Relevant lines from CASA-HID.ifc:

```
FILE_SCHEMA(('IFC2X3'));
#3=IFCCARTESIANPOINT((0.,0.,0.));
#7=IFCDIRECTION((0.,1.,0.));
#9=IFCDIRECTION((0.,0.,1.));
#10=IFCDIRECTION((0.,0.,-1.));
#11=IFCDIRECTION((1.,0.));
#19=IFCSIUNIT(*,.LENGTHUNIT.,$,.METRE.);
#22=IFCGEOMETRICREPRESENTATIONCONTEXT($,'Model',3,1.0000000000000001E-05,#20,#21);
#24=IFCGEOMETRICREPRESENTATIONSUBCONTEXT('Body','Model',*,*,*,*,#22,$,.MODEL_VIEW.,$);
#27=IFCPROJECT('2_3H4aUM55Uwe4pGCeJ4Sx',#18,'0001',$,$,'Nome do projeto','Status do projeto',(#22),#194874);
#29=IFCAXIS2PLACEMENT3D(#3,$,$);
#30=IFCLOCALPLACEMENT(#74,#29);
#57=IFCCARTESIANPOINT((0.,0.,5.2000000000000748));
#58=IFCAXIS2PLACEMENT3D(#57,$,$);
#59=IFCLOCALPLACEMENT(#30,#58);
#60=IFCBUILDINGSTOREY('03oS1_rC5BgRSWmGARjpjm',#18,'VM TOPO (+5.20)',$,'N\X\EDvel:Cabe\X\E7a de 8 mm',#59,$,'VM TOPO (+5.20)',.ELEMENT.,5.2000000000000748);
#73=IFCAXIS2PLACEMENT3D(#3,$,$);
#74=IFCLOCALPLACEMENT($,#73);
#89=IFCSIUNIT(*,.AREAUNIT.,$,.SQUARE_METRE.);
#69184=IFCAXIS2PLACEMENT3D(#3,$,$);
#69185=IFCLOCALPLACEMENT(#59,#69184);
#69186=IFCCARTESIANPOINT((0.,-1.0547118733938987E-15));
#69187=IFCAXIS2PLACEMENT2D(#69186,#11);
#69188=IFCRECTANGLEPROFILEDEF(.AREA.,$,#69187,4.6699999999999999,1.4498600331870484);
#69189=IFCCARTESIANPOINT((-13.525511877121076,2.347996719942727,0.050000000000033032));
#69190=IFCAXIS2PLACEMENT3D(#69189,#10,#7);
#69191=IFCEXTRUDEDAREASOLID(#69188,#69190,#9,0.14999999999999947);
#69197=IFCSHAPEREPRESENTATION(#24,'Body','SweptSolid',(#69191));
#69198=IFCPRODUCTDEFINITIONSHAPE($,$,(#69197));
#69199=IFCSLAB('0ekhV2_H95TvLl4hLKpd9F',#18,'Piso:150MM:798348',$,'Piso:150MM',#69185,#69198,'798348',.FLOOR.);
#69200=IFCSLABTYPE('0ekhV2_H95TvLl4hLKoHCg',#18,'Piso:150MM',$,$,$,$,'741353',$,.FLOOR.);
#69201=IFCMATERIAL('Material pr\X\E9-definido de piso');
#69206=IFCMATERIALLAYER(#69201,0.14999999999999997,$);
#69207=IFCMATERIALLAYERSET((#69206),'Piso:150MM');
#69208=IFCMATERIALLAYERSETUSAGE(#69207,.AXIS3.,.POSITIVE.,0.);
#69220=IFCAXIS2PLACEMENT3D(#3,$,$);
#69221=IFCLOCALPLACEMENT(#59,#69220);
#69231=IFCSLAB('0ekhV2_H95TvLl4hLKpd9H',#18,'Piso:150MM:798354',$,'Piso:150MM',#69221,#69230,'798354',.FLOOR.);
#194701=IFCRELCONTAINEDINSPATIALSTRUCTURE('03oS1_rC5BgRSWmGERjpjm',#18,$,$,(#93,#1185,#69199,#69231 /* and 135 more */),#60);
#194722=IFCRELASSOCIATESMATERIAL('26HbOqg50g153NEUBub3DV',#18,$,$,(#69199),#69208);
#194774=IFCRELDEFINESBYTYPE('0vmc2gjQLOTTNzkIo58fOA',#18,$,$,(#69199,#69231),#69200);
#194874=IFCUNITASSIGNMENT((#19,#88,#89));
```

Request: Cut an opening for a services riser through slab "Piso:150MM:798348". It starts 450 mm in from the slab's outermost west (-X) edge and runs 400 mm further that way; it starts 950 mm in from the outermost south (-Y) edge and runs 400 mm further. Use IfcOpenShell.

```python
import numpy as np
import ifcopenshell
import ifcopenshell.api.feature
import ifcopenshell.api.geometry
import ifcopenshell.api.root
import ifcopenshell.geom
import ifcopenshell.util.placement
import ifcopenshell.util.representation
import ifcopenshell.util.shape
import ifcopenshell.util.unit

model = ifcopenshell.open("CASA-HID.ifc")
unit_scale = ifcopenshell.util.unit.calculate_unit_scale(model)
settings = ifcopenshell.geom.settings()


def volume(element):
    """Net volume in cubic metres, openings subtracted."""
    shape = ifcopenshell.geom.create_shape(settings, element)
    return ifcopenshell.util.shape.get_volume(shape.geometry)


slab = model.by_id(69199)
before = volume(slab)

# Extent in the slab's own axes, in metres. The edges named are its -X and -Y sides.
slab_shape = ifcopenshell.geom.create_shape(settings, slab)
vertices = ifcopenshell.util.shape.get_vertices(slab_shape.geometry)
x_min, y_min, bottom = vertices.min(axis=0)
top = vertices[:, 2].max()

opening = ifcopenshell.api.root.create_entity(model, ifc_class="IfcOpeningElement", name="Services riser opening")
context = ifcopenshell.util.representation.get_context(model, "Model", "Body", "MODEL_VIEW")
width, depth = 0.4, 0.4
outline = [(0.0, 0.0), (width, 0.0), (width, depth), (0.0, depth), (0.0, 0.0)]
# Overshoot both faces by 50 mm so the cut is clean.
shape = ifcopenshell.api.geometry.add_slab_representation(
    model, context=context, depth=top - bottom + 0.1, polyline=outline
)
ifcopenshell.api.geometry.assign_representation(model, product=opening, representation=shape)

matrix = ifcopenshell.util.placement.get_local_placement(slab.ObjectPlacement)
matrix[:, 3] = matrix @ np.append(np.array([x_min + 0.45, y_min + 0.95, bottom - 0.05]) / unit_scale, 1.0)
ifcopenshell.api.geometry.edit_object_placement(model, product=opening, matrix=matrix, is_si=False)
ifcopenshell.api.feature.add_feature(model, feature=opening, element=slab)

after = volume(slab)

print(f"slab volume {before:.3f} -> {after:.3f} m3")

model.write("CASA-HID_edited.ifc")
```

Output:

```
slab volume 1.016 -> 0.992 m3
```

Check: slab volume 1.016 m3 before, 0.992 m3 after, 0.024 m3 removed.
